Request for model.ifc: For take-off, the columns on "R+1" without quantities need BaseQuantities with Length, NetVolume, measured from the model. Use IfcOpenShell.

First a look at what the model holds.

```python
import ifcopenshell
import ifcopenshell.util.element
import ifcopenshell.util.unit

model = ifcopenshell.open("model.ifc")
print(model.schema)
for unit_type in ("LENGTHUNIT", "AREAUNIT", "VOLUMEUNIT"):
    print(unit_type, ifcopenshell.util.unit.calculate_unit_scale(model, unit_type))
storey = next(s for s in model.by_type("IfcBuildingStorey") if s.Name == "R+1")
columns = [e for e in ifcopenshell.util.element.get_decomposition(storey) if e.is_a("IfcColumn")]
for e in sorted(columns, key=lambda e: e.id()):
    print(e.id(), e.is_a(), e.Name, list(ifcopenshell.util.element.get_psets(e, qtos_only=True)), sep=" | ")
```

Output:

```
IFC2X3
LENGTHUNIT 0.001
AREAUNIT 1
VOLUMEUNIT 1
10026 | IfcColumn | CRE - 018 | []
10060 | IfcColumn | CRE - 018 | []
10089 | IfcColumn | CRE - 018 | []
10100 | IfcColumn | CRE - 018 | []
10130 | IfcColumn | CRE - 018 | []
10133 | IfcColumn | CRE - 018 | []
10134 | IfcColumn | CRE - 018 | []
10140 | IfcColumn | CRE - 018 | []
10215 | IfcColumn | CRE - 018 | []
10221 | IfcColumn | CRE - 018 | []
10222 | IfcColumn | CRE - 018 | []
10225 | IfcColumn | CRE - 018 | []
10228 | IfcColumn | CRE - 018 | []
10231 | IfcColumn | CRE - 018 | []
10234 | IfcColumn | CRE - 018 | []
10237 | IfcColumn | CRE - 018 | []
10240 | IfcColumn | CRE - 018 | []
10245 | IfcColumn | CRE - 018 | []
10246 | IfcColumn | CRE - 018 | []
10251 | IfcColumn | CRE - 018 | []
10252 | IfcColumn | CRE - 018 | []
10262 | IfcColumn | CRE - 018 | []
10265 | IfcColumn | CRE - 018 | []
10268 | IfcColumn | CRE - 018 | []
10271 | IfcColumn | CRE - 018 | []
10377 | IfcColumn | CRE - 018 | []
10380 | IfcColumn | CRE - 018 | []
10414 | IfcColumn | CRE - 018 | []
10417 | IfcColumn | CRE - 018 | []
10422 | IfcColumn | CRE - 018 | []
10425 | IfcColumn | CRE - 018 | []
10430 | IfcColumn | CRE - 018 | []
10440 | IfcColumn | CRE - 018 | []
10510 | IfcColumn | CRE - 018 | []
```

```python
import ifcopenshell
import ifcopenshell.api.pset
import ifcopenshell.geom
import ifcopenshell.util.element
import ifcopenshell.util.shape
import ifcopenshell.util.unit

model = ifcopenshell.open("model.ifc")
unit_scale = ifcopenshell.util.unit.calculate_unit_scale(model)
volume_scale = ifcopenshell.util.unit.calculate_unit_scale(model, "VOLUMEUNIT")
settings = ifcopenshell.geom.settings()

storey = next(s for s in model.by_type("IfcBuildingStorey") if s.Name == "R+1")
columns = [e for e in ifcopenshell.util.element.get_decomposition(storey) if e.is_a("IfcColumn")]

for e in sorted(columns, key=lambda e: e.id()):
    if ifcopenshell.util.element.get_psets(e, qtos_only=True, should_inherit=False):
        continue
    # Geometry comes back in metres, in the element's own axes.
    shape = ifcopenshell.geom.create_shape(settings, e)
    values = {
        "Length": ifcopenshell.util.shape.get_z(shape.geometry) / unit_scale,
        "NetVolume": ifcopenshell.util.shape.get_volume(shape.geometry) / volume_scale,
    }
    qto = ifcopenshell.api.pset.add_qto(model, product=e, name="BaseQuantities")
    ifcopenshell.api.pset.edit_qto(model, qto=qto, properties=values)
    print(e.id(), {k: round(v, 3) for k, v in values.items()})

model.write("model-out.ifc")
```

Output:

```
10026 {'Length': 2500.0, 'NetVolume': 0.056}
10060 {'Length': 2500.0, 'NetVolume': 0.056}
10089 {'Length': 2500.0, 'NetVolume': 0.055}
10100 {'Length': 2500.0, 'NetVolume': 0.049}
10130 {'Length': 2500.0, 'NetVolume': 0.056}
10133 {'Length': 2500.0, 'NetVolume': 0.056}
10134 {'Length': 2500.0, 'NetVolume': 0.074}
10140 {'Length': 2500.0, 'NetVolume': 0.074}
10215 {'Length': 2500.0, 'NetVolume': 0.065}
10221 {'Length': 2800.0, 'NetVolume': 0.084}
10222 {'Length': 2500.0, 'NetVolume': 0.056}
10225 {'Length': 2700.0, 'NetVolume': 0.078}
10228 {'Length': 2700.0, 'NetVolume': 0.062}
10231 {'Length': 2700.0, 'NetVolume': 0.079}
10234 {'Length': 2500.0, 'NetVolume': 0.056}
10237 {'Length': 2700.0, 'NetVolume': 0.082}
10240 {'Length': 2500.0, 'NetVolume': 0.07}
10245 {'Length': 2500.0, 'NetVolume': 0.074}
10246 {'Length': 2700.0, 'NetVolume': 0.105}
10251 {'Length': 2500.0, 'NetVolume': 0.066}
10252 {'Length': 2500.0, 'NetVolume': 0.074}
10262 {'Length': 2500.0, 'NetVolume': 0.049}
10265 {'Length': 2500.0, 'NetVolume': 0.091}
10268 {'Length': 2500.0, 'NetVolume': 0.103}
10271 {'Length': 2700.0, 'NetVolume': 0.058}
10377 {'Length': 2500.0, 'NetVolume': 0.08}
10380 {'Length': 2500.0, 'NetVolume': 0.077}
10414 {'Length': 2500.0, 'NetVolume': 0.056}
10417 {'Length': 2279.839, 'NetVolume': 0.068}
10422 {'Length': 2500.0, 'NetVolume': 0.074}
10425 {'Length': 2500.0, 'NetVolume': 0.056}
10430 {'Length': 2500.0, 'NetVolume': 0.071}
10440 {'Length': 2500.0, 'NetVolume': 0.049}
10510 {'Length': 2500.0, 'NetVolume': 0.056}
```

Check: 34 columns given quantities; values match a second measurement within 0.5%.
